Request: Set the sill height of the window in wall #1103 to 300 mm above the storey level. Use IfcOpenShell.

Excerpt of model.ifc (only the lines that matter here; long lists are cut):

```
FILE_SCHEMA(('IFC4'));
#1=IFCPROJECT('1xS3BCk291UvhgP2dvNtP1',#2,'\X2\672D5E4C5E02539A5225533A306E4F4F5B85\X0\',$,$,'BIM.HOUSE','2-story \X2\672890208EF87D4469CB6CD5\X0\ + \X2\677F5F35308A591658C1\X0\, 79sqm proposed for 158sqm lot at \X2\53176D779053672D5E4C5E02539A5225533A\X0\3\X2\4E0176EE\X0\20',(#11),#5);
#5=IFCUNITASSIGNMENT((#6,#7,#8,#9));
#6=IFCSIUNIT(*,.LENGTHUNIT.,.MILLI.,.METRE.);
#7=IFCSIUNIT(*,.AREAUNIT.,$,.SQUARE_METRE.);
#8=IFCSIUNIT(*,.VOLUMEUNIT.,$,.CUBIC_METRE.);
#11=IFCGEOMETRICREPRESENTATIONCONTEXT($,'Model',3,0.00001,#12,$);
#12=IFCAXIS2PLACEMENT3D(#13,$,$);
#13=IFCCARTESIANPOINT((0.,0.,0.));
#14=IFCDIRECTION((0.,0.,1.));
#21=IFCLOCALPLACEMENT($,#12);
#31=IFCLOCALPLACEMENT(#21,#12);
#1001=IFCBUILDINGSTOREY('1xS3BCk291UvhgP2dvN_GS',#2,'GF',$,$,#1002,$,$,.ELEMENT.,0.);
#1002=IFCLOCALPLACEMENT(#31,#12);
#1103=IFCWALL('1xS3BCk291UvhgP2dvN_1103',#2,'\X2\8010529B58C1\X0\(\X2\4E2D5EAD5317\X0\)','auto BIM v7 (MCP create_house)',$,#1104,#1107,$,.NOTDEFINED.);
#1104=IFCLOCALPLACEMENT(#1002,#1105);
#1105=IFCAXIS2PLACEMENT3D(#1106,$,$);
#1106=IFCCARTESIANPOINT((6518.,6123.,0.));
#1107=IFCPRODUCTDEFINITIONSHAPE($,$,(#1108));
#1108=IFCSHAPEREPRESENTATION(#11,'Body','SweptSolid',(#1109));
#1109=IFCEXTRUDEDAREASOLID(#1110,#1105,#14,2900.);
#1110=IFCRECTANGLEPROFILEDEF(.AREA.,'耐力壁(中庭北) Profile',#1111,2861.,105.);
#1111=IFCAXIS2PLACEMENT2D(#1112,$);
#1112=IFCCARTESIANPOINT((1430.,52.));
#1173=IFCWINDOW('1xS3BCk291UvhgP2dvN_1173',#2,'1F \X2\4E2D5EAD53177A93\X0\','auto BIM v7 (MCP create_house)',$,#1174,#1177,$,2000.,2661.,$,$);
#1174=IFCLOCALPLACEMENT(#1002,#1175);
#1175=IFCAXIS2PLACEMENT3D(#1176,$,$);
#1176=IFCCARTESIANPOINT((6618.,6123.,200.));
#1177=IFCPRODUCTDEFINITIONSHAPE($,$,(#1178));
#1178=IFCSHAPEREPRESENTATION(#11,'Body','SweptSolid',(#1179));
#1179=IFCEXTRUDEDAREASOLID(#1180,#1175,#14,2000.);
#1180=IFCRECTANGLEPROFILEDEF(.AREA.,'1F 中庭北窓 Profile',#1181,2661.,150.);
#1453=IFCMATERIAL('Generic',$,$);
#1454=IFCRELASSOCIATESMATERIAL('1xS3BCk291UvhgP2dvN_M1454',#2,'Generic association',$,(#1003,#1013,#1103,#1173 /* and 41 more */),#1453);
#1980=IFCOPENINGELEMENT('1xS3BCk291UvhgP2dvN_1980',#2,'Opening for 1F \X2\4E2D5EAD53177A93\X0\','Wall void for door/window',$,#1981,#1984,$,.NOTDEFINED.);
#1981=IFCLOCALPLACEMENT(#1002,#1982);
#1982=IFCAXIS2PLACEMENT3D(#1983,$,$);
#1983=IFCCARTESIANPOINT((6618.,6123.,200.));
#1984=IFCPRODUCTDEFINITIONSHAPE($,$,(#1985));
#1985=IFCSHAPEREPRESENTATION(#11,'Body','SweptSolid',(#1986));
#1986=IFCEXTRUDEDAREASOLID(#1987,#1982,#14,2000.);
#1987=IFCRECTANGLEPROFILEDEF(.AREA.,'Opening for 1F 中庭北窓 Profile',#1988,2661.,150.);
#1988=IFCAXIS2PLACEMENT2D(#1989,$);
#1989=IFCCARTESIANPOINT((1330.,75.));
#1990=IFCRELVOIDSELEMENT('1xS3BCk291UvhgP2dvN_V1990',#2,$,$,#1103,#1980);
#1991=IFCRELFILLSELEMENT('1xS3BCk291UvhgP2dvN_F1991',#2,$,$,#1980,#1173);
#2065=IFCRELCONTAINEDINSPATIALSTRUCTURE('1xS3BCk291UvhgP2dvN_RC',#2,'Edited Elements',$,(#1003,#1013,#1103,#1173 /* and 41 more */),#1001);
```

```python
import numpy as np
import ifcopenshell
import ifcopenshell.api.geometry
import ifcopenshell.geom
import ifcopenshell.util.element
import ifcopenshell.util.placement
import ifcopenshell.util.shape
import ifcopenshell.util.unit

model = ifcopenshell.open("model.ifc")
unit_scale = ifcopenshell.util.unit.calculate_unit_scale(model)

window = model.by_guid("1xS3BCk291UvhgP2dvN_1173")
opening = window.FillsVoids[0].RelatingOpeningElement
storey = ifcopenshell.util.element.get_container(window, ifc_class="IfcBuildingStorey")
level = ifcopenshell.util.placement.get_local_placement(storey.ObjectPlacement)[2, 3]

# The opening's origin need not be at the sill, so measure its lowest point.
shape = ifcopenshell.geom.create_shape(ifcopenshell.geom.settings(), opening)
bottom = ifcopenshell.util.shape.get_shape_bottom_elevation(shape, shape.geometry) / unit_scale
dz = level + 300.0 - bottom

shift = np.array([0.0, 0.0, dz])
# The window is not placed relative to its opening, so move both.
for product in (opening, window):
    matrix = ifcopenshell.util.placement.get_local_placement(product.ObjectPlacement)
    matrix[:3, 3] += shift
    ifcopenshell.api.geometry.edit_object_placement(model, product=product, matrix=matrix, is_si=False)

print(f"moved by {dz * unit_scale:+.3f} m")

model.write("model_updated.ifc")
```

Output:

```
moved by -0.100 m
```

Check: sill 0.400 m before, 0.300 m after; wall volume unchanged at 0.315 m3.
